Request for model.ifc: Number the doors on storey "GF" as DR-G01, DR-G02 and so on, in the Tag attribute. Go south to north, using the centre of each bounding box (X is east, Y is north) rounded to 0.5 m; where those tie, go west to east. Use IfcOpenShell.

First a look at what the model holds.

```python
import ifcopenshell
import ifcopenshell.util.element
import ifcopenshell.util.placement

model = ifcopenshell.open("model.ifc")
print(model.schema)
storey = next(s for s in model.by_type("IfcBuildingStorey") if s.Name == "GF")
doors = [e for e in ifcopenshell.util.element.get_decomposition(storey) if e.is_a("IfcDoor")]
for e in sorted(doors, key=lambda e: e.id()):
    origin = ifcopenshell.util.placement.get_local_placement(e.ObjectPlacement)[:3, 3]
    print(e.id(), e.Tag, e.Name, origin.round(2) + 0.0, sep=" | ")
```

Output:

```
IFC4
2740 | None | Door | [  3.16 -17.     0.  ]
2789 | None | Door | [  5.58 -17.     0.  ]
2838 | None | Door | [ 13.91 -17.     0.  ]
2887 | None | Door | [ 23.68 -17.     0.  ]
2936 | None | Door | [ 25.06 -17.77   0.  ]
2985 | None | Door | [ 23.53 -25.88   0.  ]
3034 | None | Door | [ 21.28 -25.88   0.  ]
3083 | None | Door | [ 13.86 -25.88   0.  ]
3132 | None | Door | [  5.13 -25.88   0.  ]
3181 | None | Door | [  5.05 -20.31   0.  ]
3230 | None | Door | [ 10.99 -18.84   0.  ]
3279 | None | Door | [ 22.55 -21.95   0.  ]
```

```python
import ifcopenshell
import ifcopenshell.geom
import ifcopenshell.util.element
import ifcopenshell.util.shape

model = ifcopenshell.open("model.ifc")
settings = ifcopenshell.geom.settings()
settings.set("use-world-coords", True)


def centre(element):
    shape = ifcopenshell.geom.create_shape(settings, element)
    return ifcopenshell.util.shape.get_bbox_centroid(shape.geometry)


storey = next(s for s in model.by_type("IfcBuildingStorey") if s.Name == "GF")
doors = [e for e in ifcopenshell.util.element.get_decomposition(storey) if e.is_a("IfcDoor")]

# Insertion points can sit at a corner or the storey origin, so sort by the geometry (in metres).
centres = {e: centre(e) for e in doors}
doors.sort(key=lambda e: (round(centres[e][1] / 0.5), centres[e][0]))

for i, e in enumerate(doors, start=1):
    number = f"DR-G{i:02d}"
    e.Tag = number
    print(e.id(), number)

model.write("model_edited.ifc")
```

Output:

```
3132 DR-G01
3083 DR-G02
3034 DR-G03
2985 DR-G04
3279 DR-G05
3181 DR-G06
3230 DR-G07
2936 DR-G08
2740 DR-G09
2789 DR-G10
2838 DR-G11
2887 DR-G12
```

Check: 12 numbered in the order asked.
